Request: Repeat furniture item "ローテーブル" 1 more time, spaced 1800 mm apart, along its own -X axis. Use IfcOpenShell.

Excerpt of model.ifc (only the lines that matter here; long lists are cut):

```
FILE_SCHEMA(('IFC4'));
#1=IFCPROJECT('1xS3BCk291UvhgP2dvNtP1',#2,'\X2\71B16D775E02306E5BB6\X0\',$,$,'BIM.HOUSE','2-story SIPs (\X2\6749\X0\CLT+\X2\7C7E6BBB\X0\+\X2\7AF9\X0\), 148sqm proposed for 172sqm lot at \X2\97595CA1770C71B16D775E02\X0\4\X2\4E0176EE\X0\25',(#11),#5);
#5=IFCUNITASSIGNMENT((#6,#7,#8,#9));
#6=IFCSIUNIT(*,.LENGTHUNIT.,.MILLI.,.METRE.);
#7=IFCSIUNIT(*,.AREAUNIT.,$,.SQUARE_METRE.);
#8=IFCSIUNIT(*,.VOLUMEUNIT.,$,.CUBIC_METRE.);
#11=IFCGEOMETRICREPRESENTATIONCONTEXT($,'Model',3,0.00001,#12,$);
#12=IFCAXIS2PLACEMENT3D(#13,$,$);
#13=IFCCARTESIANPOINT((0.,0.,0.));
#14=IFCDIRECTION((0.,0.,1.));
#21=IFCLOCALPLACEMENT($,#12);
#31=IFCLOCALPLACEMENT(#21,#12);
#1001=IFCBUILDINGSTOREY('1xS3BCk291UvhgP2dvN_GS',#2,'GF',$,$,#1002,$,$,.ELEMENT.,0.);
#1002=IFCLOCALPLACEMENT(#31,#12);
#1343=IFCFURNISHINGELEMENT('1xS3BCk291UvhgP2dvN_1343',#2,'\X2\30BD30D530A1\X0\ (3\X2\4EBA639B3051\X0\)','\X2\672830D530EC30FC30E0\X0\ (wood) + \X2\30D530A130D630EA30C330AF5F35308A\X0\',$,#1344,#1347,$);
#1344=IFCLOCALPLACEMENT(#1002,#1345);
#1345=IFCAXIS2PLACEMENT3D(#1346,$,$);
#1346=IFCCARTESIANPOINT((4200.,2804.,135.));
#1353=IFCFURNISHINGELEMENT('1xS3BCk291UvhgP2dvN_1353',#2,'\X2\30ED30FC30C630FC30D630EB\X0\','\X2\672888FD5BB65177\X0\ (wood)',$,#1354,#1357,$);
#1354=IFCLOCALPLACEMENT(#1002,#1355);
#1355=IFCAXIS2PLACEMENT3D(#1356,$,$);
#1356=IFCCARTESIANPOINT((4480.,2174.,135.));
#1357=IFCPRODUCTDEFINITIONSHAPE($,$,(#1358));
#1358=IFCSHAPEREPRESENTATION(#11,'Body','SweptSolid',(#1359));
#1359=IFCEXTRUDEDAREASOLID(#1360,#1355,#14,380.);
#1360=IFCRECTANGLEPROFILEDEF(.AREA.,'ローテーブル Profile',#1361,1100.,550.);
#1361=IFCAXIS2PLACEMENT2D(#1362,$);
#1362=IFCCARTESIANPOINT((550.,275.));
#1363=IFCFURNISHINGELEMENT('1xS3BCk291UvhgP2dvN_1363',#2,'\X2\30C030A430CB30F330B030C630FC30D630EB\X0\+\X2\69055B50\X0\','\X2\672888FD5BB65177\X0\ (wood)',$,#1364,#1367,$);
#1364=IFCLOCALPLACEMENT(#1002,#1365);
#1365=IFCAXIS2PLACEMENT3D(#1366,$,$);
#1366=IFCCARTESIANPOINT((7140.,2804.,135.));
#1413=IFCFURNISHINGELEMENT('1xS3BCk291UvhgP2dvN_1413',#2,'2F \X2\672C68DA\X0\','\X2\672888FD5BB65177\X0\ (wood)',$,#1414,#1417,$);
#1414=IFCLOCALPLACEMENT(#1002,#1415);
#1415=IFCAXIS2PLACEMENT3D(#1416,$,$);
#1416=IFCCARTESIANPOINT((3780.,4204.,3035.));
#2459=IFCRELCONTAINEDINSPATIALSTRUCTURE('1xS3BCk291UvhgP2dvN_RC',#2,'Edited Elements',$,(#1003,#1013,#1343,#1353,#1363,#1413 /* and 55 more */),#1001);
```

```python
import ifcopenshell
import ifcopenshell.api.geometry
import ifcopenshell.api.root
import ifcopenshell.util.element
import ifcopenshell.util.placement
import ifcopenshell.util.unit

model = ifcopenshell.open("model.ifc")
unit_scale = ifcopenshell.util.unit.calculate_unit_scale(model)


def reuse_history(source, copy):
    """copy_class also copies each property set's owner history, people and application; keep the originals."""
    for rel in copy.IsDefinedBy:
        if rel.is_a("IfcRelDefinesByProperties") and (history := rel.RelatingPropertyDefinition.OwnerHistory):
            rel.RelatingPropertyDefinition.OwnerHistory = source.OwnerHistory
            ifcopenshell.util.element.remove_deep2(model, history)


source = model.by_guid("1xS3BCk291UvhgP2dvN_1353")
base = ifcopenshell.util.placement.get_local_placement(source.ObjectPlacement)
step = -base[:3, 0] * 1.8 / unit_scale

for i in range(1, 2):
    copy = ifcopenshell.api.root.copy_class(model, product=source)
    copy.Representation = ifcopenshell.util.element.copy_deep(
        model, source.Representation, exclude=["IfcGeometricRepresentationContext", "IfcRepresentationMap"]
    )
    reuse_history(source, copy)
    matrix = base.copy()
    matrix[:3, 3] += i * step
    print("added at", matrix[:3, 3].round(3) + 0.0)
    ifcopenshell.api.geometry.edit_object_placement(model, product=copy, matrix=matrix, is_si=False)

model.write("model_rev.ifc")
```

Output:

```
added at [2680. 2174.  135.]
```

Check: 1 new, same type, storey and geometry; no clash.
